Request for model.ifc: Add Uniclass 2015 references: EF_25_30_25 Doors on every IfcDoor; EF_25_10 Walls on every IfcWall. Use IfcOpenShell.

First a look at what the model holds.

```python
import ifcopenshell

model = ifcopenshell.open("model.ifc")
print(model.schema)
print("classifications:", [c.Name for c in model.by_type("IfcClassification")])
for ifc_class in ("IfcDoor", "IfcRoof", "IfcStair", "IfcWall", "IfcWindow"):
    print(ifc_class, len(model.by_type(ifc_class)))
```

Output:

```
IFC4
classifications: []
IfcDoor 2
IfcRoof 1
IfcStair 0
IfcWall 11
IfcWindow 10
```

```python
import ifcopenshell
import ifcopenshell.api.classification

model = ifcopenshell.open("model.ifc")

system = ifcopenshell.api.classification.add_classification(model, classification="Uniclass 2015")

codes = {
    "IfcDoor": ("EF_25_30_25", "Doors"),
    "IfcWall": ("EF_25_10", "Walls"),
}
for ifc_class, (code, name) in codes.items():
    products = model.by_type(ifc_class)
    ifcopenshell.api.classification.add_reference(
        model, products=products, classification=system, identification=code, name=name
    )
    print(code, len(products))

model.write("model_edited.ifc")
```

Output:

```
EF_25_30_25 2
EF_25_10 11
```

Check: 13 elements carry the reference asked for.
